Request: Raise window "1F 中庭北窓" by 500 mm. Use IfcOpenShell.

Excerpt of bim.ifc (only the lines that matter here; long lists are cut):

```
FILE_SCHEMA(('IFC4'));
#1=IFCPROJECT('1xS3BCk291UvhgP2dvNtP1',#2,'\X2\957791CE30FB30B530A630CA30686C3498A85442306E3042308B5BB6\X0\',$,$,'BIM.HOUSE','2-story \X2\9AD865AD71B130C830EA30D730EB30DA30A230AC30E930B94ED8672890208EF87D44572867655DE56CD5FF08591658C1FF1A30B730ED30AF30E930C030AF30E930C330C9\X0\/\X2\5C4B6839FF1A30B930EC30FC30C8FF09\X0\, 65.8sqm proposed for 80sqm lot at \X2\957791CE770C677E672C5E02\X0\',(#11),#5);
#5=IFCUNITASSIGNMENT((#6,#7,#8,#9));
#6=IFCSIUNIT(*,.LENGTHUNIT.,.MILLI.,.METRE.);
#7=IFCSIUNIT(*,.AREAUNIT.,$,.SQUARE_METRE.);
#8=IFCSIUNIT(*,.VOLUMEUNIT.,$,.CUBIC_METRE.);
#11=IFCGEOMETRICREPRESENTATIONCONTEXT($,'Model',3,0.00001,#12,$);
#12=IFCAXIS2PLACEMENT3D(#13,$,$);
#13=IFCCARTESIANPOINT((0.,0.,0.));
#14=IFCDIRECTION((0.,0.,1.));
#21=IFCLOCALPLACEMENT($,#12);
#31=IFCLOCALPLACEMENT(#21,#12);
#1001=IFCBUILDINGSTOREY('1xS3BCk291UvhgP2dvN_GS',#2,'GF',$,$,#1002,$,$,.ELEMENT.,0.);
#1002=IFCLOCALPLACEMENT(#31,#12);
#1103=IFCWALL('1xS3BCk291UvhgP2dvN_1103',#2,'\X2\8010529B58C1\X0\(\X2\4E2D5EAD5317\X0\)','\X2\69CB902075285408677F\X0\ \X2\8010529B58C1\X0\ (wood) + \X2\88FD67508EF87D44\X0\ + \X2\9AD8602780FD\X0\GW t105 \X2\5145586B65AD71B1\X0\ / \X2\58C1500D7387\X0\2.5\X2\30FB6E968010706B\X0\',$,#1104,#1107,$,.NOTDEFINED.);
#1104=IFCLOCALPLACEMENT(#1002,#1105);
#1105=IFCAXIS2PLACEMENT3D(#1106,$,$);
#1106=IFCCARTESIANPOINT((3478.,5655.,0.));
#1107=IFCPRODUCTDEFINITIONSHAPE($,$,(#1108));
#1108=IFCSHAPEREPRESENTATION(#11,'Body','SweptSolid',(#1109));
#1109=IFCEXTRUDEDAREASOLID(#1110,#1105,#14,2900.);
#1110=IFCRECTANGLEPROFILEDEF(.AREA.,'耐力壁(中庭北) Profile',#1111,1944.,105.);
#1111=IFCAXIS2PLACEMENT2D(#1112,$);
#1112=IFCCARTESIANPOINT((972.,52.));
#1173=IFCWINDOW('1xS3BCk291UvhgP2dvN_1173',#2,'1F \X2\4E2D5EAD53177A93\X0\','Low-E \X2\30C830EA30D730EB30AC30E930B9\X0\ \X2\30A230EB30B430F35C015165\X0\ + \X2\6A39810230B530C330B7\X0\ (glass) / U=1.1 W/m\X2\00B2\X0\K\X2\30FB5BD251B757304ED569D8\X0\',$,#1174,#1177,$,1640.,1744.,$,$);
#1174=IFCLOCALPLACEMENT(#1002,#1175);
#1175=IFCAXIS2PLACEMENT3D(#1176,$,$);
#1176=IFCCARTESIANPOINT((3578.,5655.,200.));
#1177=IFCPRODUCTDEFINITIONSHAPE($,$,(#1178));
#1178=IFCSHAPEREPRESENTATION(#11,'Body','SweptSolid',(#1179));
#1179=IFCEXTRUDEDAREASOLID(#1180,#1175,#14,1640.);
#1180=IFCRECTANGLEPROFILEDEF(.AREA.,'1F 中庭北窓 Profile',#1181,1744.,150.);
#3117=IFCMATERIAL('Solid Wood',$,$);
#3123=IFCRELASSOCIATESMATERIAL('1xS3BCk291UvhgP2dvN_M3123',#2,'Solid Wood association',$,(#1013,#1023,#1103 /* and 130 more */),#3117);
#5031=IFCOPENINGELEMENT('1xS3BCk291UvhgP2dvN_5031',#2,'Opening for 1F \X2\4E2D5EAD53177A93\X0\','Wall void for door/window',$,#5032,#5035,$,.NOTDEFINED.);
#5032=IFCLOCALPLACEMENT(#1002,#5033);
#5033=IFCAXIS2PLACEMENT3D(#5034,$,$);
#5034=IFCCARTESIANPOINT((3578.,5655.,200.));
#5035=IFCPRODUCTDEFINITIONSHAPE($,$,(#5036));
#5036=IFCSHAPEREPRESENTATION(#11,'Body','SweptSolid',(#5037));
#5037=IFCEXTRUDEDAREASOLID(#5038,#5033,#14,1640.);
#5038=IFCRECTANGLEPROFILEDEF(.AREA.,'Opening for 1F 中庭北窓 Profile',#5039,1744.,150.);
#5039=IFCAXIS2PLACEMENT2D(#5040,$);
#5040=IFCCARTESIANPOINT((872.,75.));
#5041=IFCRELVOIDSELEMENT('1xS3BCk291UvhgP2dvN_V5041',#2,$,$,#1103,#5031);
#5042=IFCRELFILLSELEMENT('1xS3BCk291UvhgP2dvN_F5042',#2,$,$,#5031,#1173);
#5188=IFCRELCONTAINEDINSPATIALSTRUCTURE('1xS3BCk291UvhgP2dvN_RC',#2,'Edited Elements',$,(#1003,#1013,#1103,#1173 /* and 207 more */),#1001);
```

```python
import numpy as np
import ifcopenshell
import ifcopenshell.api.geometry
import ifcopenshell.util.placement
import ifcopenshell.util.unit

model = ifcopenshell.open("bim.ifc")
unit_scale = ifcopenshell.util.unit.calculate_unit_scale(model)

window = model.by_guid("1xS3BCk291UvhgP2dvN_1173")
opening = window.FillsVoids[0].RelatingOpeningElement
dz = 500.0

shift = np.array([0.0, 0.0, dz])
# The window is not placed relative to its opening, so move both.
for product in (opening, window):
    matrix = ifcopenshell.util.placement.get_local_placement(product.ObjectPlacement)
    matrix[:3, 3] += shift
    ifcopenshell.api.geometry.edit_object_placement(model, product=product, matrix=matrix, is_si=False)

print(f"moved by {dz * unit_scale:+.3f} m")

model.write("bim_v2.ifc")
```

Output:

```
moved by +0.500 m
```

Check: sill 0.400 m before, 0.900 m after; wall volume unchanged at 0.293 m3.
